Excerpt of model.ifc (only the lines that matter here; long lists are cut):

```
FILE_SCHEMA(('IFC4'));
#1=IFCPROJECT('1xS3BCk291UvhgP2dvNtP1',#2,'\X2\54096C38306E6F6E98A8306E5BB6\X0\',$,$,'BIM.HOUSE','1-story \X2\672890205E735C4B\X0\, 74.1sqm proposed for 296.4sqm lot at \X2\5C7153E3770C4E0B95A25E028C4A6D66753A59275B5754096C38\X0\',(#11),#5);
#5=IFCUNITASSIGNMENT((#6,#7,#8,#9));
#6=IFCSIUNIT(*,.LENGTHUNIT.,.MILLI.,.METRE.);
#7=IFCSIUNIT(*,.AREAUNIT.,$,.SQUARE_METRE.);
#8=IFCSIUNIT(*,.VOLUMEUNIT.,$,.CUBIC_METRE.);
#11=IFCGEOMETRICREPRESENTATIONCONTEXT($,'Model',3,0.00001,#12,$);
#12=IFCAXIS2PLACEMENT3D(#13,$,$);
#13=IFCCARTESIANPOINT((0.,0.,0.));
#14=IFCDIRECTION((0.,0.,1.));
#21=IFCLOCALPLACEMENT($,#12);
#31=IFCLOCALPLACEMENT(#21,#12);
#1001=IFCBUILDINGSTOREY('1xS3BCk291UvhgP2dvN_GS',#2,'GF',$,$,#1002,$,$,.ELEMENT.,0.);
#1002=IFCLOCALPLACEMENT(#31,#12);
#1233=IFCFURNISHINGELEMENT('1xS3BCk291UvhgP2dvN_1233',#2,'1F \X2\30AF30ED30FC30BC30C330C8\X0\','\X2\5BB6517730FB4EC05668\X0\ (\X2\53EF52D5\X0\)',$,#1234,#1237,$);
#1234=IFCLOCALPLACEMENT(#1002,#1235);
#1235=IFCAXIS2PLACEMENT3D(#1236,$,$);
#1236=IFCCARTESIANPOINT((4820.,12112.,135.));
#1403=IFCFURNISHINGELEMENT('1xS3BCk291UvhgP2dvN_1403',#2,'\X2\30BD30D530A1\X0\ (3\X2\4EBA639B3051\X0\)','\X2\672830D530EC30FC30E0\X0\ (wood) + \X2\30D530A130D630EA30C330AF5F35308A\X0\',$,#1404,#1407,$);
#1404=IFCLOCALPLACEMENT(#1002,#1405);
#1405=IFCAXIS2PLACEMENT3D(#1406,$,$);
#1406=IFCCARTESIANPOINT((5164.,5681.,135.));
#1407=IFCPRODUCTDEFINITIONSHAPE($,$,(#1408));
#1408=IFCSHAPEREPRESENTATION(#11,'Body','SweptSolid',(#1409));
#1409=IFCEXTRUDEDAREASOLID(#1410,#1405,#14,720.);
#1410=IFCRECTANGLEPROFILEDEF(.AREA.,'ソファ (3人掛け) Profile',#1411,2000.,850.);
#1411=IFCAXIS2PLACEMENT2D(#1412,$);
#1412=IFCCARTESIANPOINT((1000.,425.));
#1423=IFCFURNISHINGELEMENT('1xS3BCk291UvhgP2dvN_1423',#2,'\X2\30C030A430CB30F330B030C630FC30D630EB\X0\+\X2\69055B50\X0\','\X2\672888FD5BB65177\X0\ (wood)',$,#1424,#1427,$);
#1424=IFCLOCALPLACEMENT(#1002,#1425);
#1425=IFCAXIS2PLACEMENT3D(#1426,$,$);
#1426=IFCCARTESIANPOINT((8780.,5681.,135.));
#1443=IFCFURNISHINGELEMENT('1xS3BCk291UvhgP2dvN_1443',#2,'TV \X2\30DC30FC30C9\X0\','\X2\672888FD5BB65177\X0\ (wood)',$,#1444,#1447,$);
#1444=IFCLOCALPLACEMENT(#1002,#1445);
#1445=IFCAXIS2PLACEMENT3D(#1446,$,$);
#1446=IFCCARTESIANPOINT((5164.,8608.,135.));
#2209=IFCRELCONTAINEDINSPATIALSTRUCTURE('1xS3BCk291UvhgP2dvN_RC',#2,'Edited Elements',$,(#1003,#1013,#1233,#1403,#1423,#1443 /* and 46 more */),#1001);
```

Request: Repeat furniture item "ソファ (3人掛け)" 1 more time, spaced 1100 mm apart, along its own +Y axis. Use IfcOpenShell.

```python
import ifcopenshell
import ifcopenshell.api.geometry
import ifcopenshell.api.root
import ifcopenshell.util.element
import ifcopenshell.util.placement

model = ifcopenshell.open("model.ifc")


def reuse_history(source, copy):
    """copy_class also copies each property set's owner history, people and application; keep the originals."""
    for rel in copy.IsDefinedBy:
        if rel.is_a("IfcRelDefinesByProperties") and (history := rel.RelatingPropertyDefinition.OwnerHistory):
            rel.RelatingPropertyDefinition.OwnerHistory = source.OwnerHistory
            ifcopenshell.util.element.remove_deep2(model, history)


source = model.by_id(1403)
base = ifcopenshell.util.placement.get_local_placement(source.ObjectPlacement)
step = base[:3, 1] * 1100.0

for i in range(1, 2):
    copy = ifcopenshell.api.root.copy_class(model, product=source)
    copy.Representation = ifcopenshell.util.element.copy_deep(
        model, source.Representation, exclude=["IfcGeometricRepresentationContext", "IfcRepresentationMap"]
    )
    reuse_history(source, copy)
    matrix = base.copy()
    matrix[:3, 3] += i * step
    print("added at", matrix[:3, 3].round(3) + 0.0)
    ifcopenshell.api.geometry.edit_object_placement(model, product=copy, matrix=matrix, is_si=False)

model.write("model_v2.ifc")
```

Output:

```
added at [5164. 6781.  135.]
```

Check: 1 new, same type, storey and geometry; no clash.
